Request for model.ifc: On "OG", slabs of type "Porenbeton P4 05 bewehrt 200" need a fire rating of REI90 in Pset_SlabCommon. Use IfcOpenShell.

First a look at what the model holds.

```python
import ifcopenshell
import ifcopenshell.util.element

model = ifcopenshell.open("model.ifc")
print(model.schema)
storey = next(s for s in model.by_type("IfcBuildingStorey") if s.Name == "OG")
slabs = [e for e in ifcopenshell.util.element.get_decomposition(storey) if e.is_a("IfcSlab")]
seen = {}
for e in slabs:
    element_type = ifcopenshell.util.element.get_type(e)
    key = (element_type.Name if element_type != e and element_type else None, ifcopenshell.util.element.get_pset(e, "Pset_SlabCommon", "FireRating"))
    seen[key] = seen.get(key, 0) + 1
for (name, value), count in sorted(seen.items(), key=str):
    print(count, "x", name, "|", value)
```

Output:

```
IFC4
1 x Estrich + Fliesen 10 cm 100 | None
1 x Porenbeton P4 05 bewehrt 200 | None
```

```python
import ifcopenshell
import ifcopenshell.api.pset
import ifcopenshell.util.element

model = ifcopenshell.open("model.ifc")

storey = next(s for s in model.by_type("IfcBuildingStorey") if s.Name == "OG")
slabs = [e for e in ifcopenshell.util.element.get_decomposition(storey) if e.is_a("IfcSlab")]

count = 0
for e in slabs:
    element_type = ifcopenshell.util.element.get_type(e)
    if element_type in (None, e) or element_type.Name != "Porenbeton P4 05 bewehrt 200":
        continue
    # add_pset returns the element's existing set when there is one.
    pset = ifcopenshell.api.pset.add_pset(model, product=e, name="Pset_SlabCommon")
    ifcopenshell.api.pset.edit_pset(model, pset=pset, properties={"FireRating": "REI90"})
    count += 1

print(count, "slabs updated")

model.write("model_v2.ifc")
```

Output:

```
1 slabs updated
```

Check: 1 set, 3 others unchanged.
